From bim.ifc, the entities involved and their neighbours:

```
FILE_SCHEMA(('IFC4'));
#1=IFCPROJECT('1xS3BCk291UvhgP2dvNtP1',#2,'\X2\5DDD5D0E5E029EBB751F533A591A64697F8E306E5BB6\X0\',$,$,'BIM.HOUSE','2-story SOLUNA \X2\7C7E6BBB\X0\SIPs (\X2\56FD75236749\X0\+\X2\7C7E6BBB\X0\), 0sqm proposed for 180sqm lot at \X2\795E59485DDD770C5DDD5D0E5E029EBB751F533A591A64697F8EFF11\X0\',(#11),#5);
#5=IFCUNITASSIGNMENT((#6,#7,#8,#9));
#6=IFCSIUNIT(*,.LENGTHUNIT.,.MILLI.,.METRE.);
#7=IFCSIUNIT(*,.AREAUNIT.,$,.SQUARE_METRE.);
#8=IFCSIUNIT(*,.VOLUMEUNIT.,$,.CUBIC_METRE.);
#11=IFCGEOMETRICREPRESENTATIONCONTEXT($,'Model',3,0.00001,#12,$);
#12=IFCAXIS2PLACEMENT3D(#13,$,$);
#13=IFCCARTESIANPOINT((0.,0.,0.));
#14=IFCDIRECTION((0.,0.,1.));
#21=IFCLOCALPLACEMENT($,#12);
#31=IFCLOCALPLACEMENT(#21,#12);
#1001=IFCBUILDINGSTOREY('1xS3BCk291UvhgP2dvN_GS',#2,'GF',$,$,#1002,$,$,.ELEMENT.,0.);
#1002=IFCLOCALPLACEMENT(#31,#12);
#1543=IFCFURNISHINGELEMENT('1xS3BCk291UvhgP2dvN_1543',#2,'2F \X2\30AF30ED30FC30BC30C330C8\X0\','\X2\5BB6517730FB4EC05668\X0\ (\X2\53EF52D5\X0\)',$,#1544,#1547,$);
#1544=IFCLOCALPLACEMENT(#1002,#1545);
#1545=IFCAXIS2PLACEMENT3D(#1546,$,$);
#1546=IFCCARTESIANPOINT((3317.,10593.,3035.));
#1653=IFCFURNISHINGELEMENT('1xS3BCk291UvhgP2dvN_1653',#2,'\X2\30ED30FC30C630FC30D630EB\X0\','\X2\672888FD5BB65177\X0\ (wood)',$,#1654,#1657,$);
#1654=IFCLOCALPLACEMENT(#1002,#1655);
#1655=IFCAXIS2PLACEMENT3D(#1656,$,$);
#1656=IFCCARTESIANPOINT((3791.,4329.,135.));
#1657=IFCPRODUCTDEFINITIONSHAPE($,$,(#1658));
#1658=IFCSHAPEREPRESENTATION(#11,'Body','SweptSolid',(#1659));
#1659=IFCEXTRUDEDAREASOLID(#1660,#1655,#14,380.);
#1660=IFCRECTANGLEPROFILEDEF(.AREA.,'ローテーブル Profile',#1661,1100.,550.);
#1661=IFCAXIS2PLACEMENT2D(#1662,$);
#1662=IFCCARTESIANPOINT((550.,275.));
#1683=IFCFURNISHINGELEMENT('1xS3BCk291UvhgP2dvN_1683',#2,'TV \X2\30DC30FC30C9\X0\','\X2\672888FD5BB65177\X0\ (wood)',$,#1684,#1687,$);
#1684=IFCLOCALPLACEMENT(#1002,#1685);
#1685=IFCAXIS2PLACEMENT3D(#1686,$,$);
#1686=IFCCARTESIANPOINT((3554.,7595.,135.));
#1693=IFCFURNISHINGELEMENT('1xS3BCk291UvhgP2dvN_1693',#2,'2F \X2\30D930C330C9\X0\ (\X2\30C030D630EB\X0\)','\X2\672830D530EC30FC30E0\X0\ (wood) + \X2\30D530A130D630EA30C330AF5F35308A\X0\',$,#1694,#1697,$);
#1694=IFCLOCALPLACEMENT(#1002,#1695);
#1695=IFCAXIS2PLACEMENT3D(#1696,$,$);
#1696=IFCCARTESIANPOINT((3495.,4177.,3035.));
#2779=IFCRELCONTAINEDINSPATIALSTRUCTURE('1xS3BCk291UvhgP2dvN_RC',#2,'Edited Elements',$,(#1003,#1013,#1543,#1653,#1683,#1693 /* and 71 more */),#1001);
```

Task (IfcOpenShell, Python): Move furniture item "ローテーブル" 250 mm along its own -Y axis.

```python
import ifcopenshell
import ifcopenshell.api.geometry
import ifcopenshell.util.placement

model = ifcopenshell.open("bim.ifc")

item = model.by_guid("1xS3BCk291UvhgP2dvN_1653")
matrix = ifcopenshell.util.placement.get_local_placement(item.ObjectPlacement)
matrix[:3, 3] -= matrix[:3, 1] * 250.0
ifcopenshell.api.geometry.edit_object_placement(model, product=item, matrix=matrix, is_si=False)

print(ifcopenshell.util.placement.get_local_placement(item.ObjectPlacement).round(3) + 0.0)

model.write("bim_rev.ifc")
```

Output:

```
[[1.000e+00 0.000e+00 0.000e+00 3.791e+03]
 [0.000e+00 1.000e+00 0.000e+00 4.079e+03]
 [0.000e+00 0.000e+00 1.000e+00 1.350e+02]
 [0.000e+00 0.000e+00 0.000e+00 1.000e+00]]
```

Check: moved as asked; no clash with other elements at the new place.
